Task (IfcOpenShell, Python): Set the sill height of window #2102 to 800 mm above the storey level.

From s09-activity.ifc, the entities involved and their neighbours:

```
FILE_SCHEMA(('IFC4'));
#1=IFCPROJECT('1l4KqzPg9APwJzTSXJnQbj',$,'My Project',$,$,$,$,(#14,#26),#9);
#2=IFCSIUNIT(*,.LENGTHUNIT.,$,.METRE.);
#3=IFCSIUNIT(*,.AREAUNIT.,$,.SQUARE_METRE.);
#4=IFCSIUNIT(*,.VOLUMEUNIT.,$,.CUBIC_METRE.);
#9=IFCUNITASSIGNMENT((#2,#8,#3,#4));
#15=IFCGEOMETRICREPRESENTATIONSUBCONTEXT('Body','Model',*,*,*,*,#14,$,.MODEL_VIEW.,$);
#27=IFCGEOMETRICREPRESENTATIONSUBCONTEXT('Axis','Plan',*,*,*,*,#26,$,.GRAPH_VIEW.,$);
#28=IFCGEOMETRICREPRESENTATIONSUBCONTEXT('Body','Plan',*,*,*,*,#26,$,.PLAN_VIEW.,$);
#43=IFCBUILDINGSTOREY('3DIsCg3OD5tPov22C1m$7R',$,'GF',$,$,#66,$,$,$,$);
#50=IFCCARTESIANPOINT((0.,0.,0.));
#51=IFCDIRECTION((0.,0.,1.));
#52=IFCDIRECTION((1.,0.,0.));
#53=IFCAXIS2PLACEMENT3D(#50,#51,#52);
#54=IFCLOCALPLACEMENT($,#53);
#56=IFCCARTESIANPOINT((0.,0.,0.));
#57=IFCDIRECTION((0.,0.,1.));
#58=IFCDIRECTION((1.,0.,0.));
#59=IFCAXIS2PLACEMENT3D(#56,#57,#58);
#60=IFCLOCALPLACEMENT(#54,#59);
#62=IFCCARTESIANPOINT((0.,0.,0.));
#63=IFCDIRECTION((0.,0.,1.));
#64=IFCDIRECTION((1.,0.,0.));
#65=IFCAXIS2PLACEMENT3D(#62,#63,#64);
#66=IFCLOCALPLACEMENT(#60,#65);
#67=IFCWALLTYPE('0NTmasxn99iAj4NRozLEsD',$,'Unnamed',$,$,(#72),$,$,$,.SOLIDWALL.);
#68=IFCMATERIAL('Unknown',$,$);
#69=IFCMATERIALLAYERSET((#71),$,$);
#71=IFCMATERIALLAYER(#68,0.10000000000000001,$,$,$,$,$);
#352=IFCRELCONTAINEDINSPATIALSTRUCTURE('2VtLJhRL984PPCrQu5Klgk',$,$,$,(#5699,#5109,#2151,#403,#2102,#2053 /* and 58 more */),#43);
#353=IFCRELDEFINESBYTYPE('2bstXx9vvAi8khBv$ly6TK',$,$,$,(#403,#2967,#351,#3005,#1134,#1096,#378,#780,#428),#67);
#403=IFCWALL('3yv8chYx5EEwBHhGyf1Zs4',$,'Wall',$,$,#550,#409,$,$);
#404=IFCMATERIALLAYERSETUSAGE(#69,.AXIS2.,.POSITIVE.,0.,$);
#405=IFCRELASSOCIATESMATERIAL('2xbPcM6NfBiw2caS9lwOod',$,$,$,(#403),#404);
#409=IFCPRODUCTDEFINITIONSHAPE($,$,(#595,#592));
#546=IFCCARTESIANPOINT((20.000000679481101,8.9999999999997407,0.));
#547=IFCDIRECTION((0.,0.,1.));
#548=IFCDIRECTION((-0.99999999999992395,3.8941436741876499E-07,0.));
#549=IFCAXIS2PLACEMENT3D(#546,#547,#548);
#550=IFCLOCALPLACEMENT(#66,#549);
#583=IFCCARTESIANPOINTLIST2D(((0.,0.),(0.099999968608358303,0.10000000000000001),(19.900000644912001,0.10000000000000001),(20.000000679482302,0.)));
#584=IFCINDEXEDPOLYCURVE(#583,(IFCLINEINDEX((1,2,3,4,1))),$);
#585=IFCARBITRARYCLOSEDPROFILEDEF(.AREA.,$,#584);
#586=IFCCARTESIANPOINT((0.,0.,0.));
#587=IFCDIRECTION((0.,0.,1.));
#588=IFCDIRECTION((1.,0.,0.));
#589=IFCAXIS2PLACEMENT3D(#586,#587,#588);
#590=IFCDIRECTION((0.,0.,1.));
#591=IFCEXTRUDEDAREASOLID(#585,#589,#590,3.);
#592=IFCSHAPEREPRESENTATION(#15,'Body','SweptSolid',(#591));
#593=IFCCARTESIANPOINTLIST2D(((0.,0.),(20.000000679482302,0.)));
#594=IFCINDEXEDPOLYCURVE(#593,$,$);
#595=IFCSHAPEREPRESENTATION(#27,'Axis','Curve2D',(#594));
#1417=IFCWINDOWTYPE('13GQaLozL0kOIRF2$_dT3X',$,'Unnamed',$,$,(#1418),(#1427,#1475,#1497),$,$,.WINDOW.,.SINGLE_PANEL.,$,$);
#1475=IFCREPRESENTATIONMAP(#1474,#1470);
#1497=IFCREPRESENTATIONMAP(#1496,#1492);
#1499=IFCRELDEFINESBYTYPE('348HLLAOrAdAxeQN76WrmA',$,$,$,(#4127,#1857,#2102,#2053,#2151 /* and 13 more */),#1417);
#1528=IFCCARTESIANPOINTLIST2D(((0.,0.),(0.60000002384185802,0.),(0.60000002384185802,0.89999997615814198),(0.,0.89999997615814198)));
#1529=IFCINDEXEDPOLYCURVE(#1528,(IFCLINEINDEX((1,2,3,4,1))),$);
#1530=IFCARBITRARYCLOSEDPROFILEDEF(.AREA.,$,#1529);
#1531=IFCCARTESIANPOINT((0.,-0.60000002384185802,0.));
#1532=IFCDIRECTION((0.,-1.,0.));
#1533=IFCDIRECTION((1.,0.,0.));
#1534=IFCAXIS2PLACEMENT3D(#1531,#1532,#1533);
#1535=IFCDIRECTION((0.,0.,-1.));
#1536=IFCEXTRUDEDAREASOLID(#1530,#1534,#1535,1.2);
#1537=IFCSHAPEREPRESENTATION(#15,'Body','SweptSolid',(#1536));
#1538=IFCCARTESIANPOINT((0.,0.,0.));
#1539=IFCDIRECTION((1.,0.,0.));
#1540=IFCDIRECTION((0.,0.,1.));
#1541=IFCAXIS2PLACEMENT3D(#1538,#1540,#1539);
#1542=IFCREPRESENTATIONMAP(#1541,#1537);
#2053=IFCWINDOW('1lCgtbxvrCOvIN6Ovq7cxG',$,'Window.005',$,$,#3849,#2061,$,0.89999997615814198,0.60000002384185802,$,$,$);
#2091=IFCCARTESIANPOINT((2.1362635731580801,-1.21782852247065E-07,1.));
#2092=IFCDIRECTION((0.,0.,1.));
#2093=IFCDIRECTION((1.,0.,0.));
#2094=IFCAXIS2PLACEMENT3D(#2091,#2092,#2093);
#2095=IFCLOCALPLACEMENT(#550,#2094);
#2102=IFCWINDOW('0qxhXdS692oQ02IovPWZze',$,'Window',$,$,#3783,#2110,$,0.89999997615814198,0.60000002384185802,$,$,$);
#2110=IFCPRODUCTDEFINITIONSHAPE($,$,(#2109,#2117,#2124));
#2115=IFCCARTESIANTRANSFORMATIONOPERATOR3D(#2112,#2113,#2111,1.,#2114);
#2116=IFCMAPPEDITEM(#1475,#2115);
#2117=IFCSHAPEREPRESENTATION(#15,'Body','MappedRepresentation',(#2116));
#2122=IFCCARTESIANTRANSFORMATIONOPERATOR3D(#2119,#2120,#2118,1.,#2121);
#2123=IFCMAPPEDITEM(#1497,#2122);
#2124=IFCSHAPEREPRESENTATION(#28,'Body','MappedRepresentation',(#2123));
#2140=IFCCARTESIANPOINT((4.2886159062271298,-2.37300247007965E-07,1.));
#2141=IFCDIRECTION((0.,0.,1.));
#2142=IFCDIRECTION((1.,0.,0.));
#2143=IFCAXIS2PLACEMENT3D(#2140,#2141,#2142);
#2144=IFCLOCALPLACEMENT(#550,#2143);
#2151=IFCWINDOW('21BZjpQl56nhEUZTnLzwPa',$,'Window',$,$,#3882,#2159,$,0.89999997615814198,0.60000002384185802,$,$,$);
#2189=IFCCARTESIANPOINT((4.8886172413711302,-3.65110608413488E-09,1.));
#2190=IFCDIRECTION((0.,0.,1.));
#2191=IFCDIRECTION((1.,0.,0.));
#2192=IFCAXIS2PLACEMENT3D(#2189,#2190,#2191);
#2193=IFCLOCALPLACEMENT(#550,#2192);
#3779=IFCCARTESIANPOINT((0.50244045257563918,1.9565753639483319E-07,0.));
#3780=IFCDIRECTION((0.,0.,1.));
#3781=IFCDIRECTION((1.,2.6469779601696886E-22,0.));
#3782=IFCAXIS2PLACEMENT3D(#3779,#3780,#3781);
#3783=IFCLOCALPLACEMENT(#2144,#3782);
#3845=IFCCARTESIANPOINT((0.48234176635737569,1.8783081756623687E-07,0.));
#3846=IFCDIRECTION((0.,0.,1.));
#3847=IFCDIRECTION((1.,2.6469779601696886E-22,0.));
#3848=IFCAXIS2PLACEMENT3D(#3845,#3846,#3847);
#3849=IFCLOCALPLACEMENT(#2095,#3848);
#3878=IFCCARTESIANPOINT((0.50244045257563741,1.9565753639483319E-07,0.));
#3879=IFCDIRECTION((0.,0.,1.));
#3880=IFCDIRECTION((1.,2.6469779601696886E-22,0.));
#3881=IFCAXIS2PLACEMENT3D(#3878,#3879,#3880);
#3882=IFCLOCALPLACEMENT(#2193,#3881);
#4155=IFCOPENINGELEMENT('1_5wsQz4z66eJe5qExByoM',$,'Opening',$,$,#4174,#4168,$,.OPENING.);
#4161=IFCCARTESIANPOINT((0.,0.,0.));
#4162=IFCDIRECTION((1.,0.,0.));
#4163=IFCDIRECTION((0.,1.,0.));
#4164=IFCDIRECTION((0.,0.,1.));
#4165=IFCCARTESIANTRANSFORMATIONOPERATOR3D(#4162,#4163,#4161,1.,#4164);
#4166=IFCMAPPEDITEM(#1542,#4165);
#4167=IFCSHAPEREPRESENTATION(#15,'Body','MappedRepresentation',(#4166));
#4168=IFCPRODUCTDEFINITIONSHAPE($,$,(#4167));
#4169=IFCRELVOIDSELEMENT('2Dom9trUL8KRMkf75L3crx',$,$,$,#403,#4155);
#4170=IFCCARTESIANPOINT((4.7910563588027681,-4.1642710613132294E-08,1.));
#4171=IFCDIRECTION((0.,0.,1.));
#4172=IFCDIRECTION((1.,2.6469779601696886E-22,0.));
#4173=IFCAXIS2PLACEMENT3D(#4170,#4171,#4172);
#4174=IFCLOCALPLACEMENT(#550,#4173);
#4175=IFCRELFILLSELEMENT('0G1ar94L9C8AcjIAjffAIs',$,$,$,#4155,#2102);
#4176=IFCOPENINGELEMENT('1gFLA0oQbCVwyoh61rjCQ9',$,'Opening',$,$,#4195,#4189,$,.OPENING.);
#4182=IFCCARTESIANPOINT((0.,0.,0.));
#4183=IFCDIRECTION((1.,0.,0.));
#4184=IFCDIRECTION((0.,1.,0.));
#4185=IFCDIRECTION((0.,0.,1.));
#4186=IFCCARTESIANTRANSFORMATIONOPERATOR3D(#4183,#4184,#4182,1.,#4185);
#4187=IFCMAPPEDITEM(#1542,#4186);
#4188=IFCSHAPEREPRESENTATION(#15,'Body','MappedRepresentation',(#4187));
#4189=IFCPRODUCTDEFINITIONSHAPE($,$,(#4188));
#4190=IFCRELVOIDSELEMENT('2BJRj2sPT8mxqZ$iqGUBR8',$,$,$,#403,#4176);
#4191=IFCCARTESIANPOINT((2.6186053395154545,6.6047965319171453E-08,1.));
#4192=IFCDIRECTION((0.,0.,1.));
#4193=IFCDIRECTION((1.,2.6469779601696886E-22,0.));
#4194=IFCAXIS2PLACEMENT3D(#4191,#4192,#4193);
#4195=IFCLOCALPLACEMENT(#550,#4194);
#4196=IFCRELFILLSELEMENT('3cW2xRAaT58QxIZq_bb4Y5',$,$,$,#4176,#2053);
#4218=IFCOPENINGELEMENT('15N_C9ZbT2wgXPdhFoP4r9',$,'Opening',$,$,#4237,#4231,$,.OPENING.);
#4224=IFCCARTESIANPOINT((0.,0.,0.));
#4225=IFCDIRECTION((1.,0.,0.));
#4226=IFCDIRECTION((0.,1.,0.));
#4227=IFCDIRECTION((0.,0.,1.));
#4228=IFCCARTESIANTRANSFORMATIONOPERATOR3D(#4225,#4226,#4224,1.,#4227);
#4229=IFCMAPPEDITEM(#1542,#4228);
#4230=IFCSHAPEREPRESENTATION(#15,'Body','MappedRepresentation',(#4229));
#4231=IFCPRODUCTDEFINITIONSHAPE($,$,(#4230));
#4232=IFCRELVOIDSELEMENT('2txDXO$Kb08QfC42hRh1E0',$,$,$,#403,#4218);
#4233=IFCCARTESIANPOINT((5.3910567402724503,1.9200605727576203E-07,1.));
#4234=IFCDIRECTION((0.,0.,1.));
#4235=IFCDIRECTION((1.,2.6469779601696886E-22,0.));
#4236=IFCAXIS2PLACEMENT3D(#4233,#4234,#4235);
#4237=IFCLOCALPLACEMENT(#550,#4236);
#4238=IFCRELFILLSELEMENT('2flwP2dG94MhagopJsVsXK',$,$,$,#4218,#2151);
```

```python
import numpy as np
import ifcopenshell
import ifcopenshell.api.geometry
import ifcopenshell.geom
import ifcopenshell.util.element
import ifcopenshell.util.placement
import ifcopenshell.util.shape
import ifcopenshell.util.unit

model = ifcopenshell.open("s09-activity.ifc")
unit_scale = ifcopenshell.util.unit.calculate_unit_scale(model)

window = model.by_guid("0qxhXdS692oQ02IovPWZze")
opening = window.FillsVoids[0].RelatingOpeningElement
storey = ifcopenshell.util.element.get_container(window, ifc_class="IfcBuildingStorey")
level = ifcopenshell.util.placement.get_local_placement(storey.ObjectPlacement)[2, 3]

# The opening's origin need not be at the sill, so measure its lowest point.
shape = ifcopenshell.geom.create_shape(ifcopenshell.geom.settings(), opening)
bottom = ifcopenshell.util.shape.get_shape_bottom_elevation(shape, shape.geometry) / unit_scale
dz = level + 0.8 - bottom

shift = np.array([0.0, 0.0, dz])
# The window is not placed relative to its opening, so move both.
for product in (opening, window):
    matrix = ifcopenshell.util.placement.get_local_placement(product.ObjectPlacement)
    matrix[:3, 3] += shift
    ifcopenshell.api.geometry.edit_object_placement(model, product=product, matrix=matrix, is_si=False)

print(f"moved by {dz * unit_scale:+.3f} m")

model.write("s09-activity_edited.ifc")
```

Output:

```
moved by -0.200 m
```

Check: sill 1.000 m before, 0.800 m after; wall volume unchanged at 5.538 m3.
